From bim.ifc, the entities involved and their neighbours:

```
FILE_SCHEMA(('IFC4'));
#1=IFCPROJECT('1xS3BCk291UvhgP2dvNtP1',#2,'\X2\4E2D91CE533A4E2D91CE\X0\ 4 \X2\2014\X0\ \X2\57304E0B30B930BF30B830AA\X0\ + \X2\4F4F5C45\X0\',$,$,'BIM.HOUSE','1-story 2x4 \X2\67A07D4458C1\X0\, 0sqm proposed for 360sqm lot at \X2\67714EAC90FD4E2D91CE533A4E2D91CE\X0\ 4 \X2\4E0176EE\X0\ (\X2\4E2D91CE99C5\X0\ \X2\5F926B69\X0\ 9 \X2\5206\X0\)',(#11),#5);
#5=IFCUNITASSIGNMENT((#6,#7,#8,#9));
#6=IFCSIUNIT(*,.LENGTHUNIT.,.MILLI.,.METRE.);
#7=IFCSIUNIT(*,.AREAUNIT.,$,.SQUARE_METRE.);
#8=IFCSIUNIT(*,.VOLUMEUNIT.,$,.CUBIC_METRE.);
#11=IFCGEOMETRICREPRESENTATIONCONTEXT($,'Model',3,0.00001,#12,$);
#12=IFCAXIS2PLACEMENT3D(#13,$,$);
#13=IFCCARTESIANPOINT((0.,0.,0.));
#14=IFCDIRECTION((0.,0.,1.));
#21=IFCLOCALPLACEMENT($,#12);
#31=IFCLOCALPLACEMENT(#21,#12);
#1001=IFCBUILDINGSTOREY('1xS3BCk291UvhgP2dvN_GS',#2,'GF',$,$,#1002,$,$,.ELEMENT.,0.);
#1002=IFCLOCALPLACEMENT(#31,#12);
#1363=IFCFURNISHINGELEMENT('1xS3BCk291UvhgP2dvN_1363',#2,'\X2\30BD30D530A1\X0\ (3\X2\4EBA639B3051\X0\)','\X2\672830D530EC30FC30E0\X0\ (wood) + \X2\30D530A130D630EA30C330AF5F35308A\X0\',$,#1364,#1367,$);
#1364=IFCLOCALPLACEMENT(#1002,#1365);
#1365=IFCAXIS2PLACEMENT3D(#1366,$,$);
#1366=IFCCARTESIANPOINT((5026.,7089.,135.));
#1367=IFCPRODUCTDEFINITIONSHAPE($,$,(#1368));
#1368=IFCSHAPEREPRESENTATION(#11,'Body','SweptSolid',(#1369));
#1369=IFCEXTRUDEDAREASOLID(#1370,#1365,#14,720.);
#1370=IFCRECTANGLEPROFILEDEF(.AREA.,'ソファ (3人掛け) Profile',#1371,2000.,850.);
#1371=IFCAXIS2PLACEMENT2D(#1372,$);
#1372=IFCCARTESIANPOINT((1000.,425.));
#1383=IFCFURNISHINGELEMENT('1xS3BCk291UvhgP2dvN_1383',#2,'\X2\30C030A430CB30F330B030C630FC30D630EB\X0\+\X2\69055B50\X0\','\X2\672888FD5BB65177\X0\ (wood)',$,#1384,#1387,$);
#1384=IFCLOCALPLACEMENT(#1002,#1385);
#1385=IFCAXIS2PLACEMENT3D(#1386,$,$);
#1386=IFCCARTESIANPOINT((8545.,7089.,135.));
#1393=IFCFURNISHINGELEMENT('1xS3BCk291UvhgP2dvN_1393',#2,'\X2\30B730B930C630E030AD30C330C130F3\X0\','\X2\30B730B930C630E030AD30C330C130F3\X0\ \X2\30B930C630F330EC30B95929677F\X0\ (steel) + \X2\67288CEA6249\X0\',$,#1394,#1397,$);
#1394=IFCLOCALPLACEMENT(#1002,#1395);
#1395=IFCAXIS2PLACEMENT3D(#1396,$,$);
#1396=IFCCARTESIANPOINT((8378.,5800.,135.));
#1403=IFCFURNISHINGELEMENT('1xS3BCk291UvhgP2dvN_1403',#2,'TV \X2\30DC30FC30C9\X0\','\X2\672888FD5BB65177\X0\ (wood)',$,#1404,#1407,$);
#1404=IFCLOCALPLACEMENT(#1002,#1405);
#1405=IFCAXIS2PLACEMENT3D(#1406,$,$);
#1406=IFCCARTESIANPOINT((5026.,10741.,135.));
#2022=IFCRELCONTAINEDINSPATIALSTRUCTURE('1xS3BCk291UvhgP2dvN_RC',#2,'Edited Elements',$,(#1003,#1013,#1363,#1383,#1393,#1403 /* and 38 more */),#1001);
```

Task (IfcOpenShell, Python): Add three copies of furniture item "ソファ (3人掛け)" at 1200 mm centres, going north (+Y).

```python
import numpy as np
import ifcopenshell
import ifcopenshell.api.geometry
import ifcopenshell.api.root
import ifcopenshell.util.element
import ifcopenshell.util.placement
import ifcopenshell.util.unit

model = ifcopenshell.open("bim.ifc")
unit_scale = ifcopenshell.util.unit.calculate_unit_scale(model)


def reuse_history(source, copy):
    """copy_class also copies each property set's owner history, people and application; keep the originals."""
    for rel in copy.IsDefinedBy:
        if rel.is_a("IfcRelDefinesByProperties") and (history := rel.RelatingPropertyDefinition.OwnerHistory):
            rel.RelatingPropertyDefinition.OwnerHistory = source.OwnerHistory
            ifcopenshell.util.element.remove_deep2(model, history)


source = model.by_guid("1xS3BCk291UvhgP2dvN_1363")
base = ifcopenshell.util.placement.get_local_placement(source.ObjectPlacement)
step = np.array([0.0, 1.0, 0.0]) * 1.2 / unit_scale

for i in range(1, 4):
    copy = ifcopenshell.api.root.copy_class(model, product=source)
    copy.Representation = ifcopenshell.util.element.copy_deep(
        model, source.Representation, exclude=["IfcGeometricRepresentationContext", "IfcRepresentationMap"]
    )
    reuse_history(source, copy)
    matrix = base.copy()
    matrix[:3, 3] += i * step
    print("added at", matrix[:3, 3].round(3) + 0.0)
    ifcopenshell.api.geometry.edit_object_placement(model, product=copy, matrix=matrix, is_si=False)

model.write("bim_v2.ifc")
```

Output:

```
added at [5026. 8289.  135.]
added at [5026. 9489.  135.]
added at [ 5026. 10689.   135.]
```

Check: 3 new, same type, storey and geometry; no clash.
